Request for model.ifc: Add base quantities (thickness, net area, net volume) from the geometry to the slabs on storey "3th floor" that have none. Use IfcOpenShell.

First a look at what the model holds.

```python
import ifcopenshell
import ifcopenshell.util.element
import ifcopenshell.util.unit

model = ifcopenshell.open("model.ifc")
print(model.schema)
for unit_type in ("LENGTHUNIT", "AREAUNIT", "VOLUMEUNIT"):
    print(unit_type, ifcopenshell.util.unit.calculate_unit_scale(model, unit_type))
storey = next(s for s in model.by_type("IfcBuildingStorey") if s.Name == "3th floor")
slabs = [e for e in ifcopenshell.util.element.get_decomposition(storey) if e.is_a("IfcSlab")]
for e in sorted(slabs, key=lambda e: e.id()):
    print(e.id(), e.is_a(), e.Name, list(ifcopenshell.util.element.get_psets(e, qtos_only=True)), sep=" | ")
```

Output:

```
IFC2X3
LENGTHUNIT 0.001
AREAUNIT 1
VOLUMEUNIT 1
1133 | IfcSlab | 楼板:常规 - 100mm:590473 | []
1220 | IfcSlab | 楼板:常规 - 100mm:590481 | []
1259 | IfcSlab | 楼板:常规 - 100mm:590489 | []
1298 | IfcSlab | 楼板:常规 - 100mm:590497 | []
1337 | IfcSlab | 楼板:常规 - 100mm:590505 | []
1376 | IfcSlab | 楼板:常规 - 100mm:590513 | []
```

```python
import ifcopenshell
import ifcopenshell.api.pset
import ifcopenshell.geom
import ifcopenshell.util.element
import ifcopenshell.util.shape
import ifcopenshell.util.unit

model = ifcopenshell.open("model.ifc")
unit_scale = ifcopenshell.util.unit.calculate_unit_scale(model)
area_scale = ifcopenshell.util.unit.calculate_unit_scale(model, "AREAUNIT")
volume_scale = ifcopenshell.util.unit.calculate_unit_scale(model, "VOLUMEUNIT")
settings = ifcopenshell.geom.settings()

storey = next(s for s in model.by_type("IfcBuildingStorey") if s.Name == "3th floor")
slabs = [e for e in ifcopenshell.util.element.get_decomposition(storey) if e.is_a("IfcSlab")]

for e in sorted(slabs, key=lambda e: e.id()):
    if ifcopenshell.util.element.get_psets(e, qtos_only=True, should_inherit=False):
        continue
    # Geometry comes back in metres, in the element's own axes.
    shape = ifcopenshell.geom.create_shape(settings, e)
    values = {
        "Width": ifcopenshell.util.shape.get_z(shape.geometry) / unit_scale,
        "NetArea": ifcopenshell.util.shape.get_footprint_area(shape.geometry) / area_scale,
        "NetVolume": ifcopenshell.util.shape.get_volume(shape.geometry) / volume_scale,
    }
    qto = ifcopenshell.api.pset.add_qto(model, product=e, name="BaseQuantities")
    ifcopenshell.api.pset.edit_qto(model, qto=qto, properties=values)
    print(e.id(), {k: round(v, 3) for k, v in values.items()})

model.write("model_rev.ifc")
```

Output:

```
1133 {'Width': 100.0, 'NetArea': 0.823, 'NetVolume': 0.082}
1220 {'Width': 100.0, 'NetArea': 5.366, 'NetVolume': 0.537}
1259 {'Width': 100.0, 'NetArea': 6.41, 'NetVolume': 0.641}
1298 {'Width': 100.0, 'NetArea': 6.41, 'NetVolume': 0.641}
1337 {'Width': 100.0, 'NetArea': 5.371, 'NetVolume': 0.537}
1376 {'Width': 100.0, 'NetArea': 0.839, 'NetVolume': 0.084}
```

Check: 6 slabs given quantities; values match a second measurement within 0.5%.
